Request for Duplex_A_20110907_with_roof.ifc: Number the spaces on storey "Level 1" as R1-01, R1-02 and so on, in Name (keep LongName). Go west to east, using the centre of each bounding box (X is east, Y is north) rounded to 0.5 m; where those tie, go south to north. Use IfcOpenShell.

First a look at what the model holds.

```python
import ifcopenshell
import ifcopenshell.util.element
import ifcopenshell.util.placement

model = ifcopenshell.open("Duplex_A_20110907_with_roof.ifc")
print(model.schema)
storey = next(s for s in model.by_type("IfcBuildingStorey") if s.Name == "Level 1")
spaces = [e for e in ifcopenshell.util.element.get_decomposition(storey) if e.is_a("IfcSpace")]
for e in sorted(spaces, key=lambda e: e.id()):
    origin = ifcopenshell.util.placement.get_local_placement(e.ObjectPlacement)[:3, 3]
    print(e.id(), e.Name, e.LongName, origin.round(2) + 0.0, sep=" | ")
```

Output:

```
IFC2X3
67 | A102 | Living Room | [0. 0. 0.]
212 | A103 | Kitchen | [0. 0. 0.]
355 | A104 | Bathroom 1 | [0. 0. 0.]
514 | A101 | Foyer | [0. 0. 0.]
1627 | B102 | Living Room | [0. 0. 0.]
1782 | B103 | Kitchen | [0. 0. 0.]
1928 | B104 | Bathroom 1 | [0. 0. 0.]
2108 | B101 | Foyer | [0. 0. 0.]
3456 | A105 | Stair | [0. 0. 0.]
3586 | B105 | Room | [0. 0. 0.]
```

```python
import ifcopenshell
import ifcopenshell.geom
import ifcopenshell.util.element
import ifcopenshell.util.shape

model = ifcopenshell.open("Duplex_A_20110907_with_roof.ifc")
settings = ifcopenshell.geom.settings()
settings.set("use-world-coords", True)


def centre(element):
    shape = ifcopenshell.geom.create_shape(settings, element)
    return ifcopenshell.util.shape.get_bbox_centroid(shape.geometry)


storey = next(s for s in model.by_type("IfcBuildingStorey") if s.Name == "Level 1")
spaces = [e for e in ifcopenshell.util.element.get_decomposition(storey) if e.is_a("IfcSpace")]

# Insertion points can sit at a corner or the storey origin, so sort by the geometry (in metres).
centres = {e: centre(e) for e in spaces}
spaces.sort(key=lambda e: (round(centres[e][0] / 0.5), centres[e][1]))

for i, e in enumerate(spaces, start=1):
    number = f"R1-{i:02d}"
    e.Name = number
    print(e.id(), number)

model.write("Duplex_A_20110907_with_roof-out.ifc")
```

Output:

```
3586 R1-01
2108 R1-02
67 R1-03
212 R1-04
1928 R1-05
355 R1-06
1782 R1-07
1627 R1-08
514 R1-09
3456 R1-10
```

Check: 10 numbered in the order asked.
